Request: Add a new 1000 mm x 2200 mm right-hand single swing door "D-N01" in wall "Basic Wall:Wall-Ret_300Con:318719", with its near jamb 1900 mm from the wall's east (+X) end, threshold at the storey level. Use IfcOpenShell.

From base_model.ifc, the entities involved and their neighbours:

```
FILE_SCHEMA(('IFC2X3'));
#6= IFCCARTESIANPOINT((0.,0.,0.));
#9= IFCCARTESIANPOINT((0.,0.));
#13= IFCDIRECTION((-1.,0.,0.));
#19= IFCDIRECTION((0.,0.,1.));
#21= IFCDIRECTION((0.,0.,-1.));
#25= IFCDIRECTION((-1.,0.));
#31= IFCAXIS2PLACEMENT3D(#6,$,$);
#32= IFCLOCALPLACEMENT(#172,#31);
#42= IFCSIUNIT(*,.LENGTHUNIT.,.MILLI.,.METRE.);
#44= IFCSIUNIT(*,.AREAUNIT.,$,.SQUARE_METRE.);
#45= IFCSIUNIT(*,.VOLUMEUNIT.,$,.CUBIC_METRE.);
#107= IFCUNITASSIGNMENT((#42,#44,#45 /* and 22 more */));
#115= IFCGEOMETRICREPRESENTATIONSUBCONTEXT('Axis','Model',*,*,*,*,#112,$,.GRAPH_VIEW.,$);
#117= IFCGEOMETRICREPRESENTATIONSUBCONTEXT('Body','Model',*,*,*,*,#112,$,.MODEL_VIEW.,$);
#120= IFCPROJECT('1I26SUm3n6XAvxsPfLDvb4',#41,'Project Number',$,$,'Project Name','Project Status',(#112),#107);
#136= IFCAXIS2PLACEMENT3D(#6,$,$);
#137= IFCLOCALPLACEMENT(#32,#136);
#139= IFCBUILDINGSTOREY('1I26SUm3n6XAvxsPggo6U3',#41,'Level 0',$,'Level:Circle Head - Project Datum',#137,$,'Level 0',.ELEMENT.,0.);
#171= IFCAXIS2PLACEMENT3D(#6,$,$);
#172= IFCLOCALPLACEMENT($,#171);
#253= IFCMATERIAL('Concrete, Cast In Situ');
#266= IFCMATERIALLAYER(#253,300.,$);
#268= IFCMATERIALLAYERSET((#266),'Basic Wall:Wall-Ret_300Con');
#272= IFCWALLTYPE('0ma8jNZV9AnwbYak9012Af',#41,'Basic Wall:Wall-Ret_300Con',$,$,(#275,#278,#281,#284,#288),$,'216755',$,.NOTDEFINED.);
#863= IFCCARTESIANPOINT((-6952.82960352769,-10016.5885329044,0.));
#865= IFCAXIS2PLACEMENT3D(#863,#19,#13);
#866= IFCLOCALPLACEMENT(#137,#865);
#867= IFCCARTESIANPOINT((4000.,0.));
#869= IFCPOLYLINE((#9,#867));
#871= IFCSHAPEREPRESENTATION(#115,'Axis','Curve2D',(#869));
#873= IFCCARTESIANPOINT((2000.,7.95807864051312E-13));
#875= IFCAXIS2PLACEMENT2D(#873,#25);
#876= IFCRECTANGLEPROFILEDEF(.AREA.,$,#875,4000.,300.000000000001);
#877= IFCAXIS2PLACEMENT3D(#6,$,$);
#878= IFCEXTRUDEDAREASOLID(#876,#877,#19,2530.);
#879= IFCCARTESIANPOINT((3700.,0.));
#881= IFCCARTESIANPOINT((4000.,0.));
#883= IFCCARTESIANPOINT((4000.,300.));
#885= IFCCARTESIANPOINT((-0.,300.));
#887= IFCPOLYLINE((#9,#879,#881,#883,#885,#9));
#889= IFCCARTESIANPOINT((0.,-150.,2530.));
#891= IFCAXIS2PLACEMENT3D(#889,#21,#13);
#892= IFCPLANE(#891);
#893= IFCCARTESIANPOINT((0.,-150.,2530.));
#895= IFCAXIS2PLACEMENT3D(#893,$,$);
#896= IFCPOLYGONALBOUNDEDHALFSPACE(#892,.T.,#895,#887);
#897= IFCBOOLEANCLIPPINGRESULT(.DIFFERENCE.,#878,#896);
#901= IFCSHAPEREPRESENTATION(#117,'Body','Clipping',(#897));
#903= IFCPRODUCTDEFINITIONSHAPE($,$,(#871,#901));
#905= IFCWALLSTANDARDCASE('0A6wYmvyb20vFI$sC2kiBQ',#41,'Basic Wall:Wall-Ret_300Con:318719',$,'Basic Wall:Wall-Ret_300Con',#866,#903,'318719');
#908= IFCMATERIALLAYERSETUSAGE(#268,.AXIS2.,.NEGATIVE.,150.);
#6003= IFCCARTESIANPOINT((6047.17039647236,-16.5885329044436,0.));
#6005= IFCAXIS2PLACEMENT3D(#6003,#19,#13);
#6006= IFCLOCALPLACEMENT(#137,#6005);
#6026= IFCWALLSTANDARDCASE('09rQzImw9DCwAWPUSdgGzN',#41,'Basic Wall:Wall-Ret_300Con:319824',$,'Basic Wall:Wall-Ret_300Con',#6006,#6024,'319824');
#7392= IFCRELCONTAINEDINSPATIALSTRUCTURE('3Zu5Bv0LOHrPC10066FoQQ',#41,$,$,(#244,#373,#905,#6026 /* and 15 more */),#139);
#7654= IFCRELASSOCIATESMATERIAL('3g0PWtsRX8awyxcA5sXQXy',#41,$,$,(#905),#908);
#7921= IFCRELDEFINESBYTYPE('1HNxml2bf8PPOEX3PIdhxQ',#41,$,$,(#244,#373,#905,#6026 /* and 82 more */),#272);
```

```python
import numpy as np
import ifcopenshell
import ifcopenshell.api.feature
import ifcopenshell.api.geometry
import ifcopenshell.api.root
import ifcopenshell.api.spatial
import ifcopenshell.api.type
import ifcopenshell.geom
import ifcopenshell.util.element
import ifcopenshell.util.placement
import ifcopenshell.util.representation
import ifcopenshell.util.shape
import ifcopenshell.util.unit

model = ifcopenshell.open("base_model.ifc")
unit_scale = ifcopenshell.util.unit.calculate_unit_scale(model)
settings = ifcopenshell.geom.settings()


def volume(element):
    """Net volume in cubic metres, openings subtracted."""
    shape = ifcopenshell.geom.create_shape(settings, element)
    return ifcopenshell.util.shape.get_volume(shape.geometry)


wall = model.by_guid("0A6wYmvyb20vFI$sC2kiBQ")
storey = ifcopenshell.util.element.get_container(wall, ifc_class="IfcBuildingStorey")
context = ifcopenshell.util.representation.get_context(model, "Model", "Body", "MODEL_VIEW")
before = volume(wall)

width, height, from_end, sill = 1, 2.2, 1.9, 0.0  # metres

# The wall runs along its own X axis, and the end named is its -X end.
wall_shape = ifcopenshell.geom.create_shape(settings, wall)
x, y, z = ifcopenshell.util.shape.get_vertices(wall_shape.geometry).T
start = x.min() + from_end
face, thickness = float(y.min()), float(y.max() - y.min())
wall_matrix = ifcopenshell.util.placement.get_local_placement(wall.ObjectPlacement)
level = ifcopenshell.util.placement.get_local_placement(storey.ObjectPlacement)[2, 3]


def in_wall(x, y):
    """Placement at x, y metres in the wall's axes, at sill height."""
    matrix = wall_matrix.copy()
    matrix[:, 3] = wall_matrix @ np.array([x / unit_scale, y / unit_scale, 0.0, 1.0])
    matrix[2, 3] = level + sill / unit_scale
    return matrix


# Opening: a box that overshoots both wall faces by 50 mm.
opening = ifcopenshell.api.root.create_entity(model, ifc_class="IfcOpeningElement")
box = ifcopenshell.api.geometry.add_wall_representation(
    model, context=context, length=width, height=height, thickness=thickness + 0.1
)
ifcopenshell.api.geometry.assign_representation(model, product=opening, representation=box)
ifcopenshell.api.geometry.edit_object_placement(model, product=opening, matrix=in_wall(start, face - 0.05), is_si=False)
ifcopenshell.api.feature.add_feature(model, feature=opening, element=wall)

door = ifcopenshell.api.root.create_entity(model, ifc_class="IfcDoor", name="D-N01")
door.OverallWidth, door.OverallHeight = width / unit_scale, height / unit_scale
body = ifcopenshell.api.geometry.add_door_representation(
    model,
    context=context,
    overall_width=door.OverallWidth,
    overall_height=door.OverallHeight,
    operation_type="SINGLE_SWING_RIGHT",
    lining_properties={"LiningDepth": thickness / unit_scale, "ThresholdDepth": thickness / unit_scale},
)
ifcopenshell.api.geometry.assign_representation(model, product=door, representation=body)
ifcopenshell.api.spatial.assign_container(model, products=[door], relating_structure=storey)
fills = ifcopenshell.api.feature.add_filling(model, opening=opening, element=door)
fills.OwnerHistory = door.OwnerHistory  # required in IFC2X3

# IFC2X3 keeps the operation on the door style.
style = ifcopenshell.api.root.create_entity(model, ifc_class="IfcDoorStyle", name="D-N01")
style.OperationType, style.ConstructionType = "SINGLE_SWING_RIGHT", "NOTDEFINED"
style.ParameterTakesPrecedence = style.Sizeable = False
ifcopenshell.api.type.assign_type(model, related_objects=[door], relating_type=style)

# The lining spans the wall, so the door starts at the wall face.
ifcopenshell.api.geometry.edit_object_placement(model, product=door, matrix=in_wall(start, face), is_si=False)

after = volume(wall)

print(f"wall volume {before:.3f} -> {after:.3f} m3")

model.write("base_model_updated.ifc")
```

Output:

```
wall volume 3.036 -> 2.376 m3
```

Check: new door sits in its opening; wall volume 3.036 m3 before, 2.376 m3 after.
